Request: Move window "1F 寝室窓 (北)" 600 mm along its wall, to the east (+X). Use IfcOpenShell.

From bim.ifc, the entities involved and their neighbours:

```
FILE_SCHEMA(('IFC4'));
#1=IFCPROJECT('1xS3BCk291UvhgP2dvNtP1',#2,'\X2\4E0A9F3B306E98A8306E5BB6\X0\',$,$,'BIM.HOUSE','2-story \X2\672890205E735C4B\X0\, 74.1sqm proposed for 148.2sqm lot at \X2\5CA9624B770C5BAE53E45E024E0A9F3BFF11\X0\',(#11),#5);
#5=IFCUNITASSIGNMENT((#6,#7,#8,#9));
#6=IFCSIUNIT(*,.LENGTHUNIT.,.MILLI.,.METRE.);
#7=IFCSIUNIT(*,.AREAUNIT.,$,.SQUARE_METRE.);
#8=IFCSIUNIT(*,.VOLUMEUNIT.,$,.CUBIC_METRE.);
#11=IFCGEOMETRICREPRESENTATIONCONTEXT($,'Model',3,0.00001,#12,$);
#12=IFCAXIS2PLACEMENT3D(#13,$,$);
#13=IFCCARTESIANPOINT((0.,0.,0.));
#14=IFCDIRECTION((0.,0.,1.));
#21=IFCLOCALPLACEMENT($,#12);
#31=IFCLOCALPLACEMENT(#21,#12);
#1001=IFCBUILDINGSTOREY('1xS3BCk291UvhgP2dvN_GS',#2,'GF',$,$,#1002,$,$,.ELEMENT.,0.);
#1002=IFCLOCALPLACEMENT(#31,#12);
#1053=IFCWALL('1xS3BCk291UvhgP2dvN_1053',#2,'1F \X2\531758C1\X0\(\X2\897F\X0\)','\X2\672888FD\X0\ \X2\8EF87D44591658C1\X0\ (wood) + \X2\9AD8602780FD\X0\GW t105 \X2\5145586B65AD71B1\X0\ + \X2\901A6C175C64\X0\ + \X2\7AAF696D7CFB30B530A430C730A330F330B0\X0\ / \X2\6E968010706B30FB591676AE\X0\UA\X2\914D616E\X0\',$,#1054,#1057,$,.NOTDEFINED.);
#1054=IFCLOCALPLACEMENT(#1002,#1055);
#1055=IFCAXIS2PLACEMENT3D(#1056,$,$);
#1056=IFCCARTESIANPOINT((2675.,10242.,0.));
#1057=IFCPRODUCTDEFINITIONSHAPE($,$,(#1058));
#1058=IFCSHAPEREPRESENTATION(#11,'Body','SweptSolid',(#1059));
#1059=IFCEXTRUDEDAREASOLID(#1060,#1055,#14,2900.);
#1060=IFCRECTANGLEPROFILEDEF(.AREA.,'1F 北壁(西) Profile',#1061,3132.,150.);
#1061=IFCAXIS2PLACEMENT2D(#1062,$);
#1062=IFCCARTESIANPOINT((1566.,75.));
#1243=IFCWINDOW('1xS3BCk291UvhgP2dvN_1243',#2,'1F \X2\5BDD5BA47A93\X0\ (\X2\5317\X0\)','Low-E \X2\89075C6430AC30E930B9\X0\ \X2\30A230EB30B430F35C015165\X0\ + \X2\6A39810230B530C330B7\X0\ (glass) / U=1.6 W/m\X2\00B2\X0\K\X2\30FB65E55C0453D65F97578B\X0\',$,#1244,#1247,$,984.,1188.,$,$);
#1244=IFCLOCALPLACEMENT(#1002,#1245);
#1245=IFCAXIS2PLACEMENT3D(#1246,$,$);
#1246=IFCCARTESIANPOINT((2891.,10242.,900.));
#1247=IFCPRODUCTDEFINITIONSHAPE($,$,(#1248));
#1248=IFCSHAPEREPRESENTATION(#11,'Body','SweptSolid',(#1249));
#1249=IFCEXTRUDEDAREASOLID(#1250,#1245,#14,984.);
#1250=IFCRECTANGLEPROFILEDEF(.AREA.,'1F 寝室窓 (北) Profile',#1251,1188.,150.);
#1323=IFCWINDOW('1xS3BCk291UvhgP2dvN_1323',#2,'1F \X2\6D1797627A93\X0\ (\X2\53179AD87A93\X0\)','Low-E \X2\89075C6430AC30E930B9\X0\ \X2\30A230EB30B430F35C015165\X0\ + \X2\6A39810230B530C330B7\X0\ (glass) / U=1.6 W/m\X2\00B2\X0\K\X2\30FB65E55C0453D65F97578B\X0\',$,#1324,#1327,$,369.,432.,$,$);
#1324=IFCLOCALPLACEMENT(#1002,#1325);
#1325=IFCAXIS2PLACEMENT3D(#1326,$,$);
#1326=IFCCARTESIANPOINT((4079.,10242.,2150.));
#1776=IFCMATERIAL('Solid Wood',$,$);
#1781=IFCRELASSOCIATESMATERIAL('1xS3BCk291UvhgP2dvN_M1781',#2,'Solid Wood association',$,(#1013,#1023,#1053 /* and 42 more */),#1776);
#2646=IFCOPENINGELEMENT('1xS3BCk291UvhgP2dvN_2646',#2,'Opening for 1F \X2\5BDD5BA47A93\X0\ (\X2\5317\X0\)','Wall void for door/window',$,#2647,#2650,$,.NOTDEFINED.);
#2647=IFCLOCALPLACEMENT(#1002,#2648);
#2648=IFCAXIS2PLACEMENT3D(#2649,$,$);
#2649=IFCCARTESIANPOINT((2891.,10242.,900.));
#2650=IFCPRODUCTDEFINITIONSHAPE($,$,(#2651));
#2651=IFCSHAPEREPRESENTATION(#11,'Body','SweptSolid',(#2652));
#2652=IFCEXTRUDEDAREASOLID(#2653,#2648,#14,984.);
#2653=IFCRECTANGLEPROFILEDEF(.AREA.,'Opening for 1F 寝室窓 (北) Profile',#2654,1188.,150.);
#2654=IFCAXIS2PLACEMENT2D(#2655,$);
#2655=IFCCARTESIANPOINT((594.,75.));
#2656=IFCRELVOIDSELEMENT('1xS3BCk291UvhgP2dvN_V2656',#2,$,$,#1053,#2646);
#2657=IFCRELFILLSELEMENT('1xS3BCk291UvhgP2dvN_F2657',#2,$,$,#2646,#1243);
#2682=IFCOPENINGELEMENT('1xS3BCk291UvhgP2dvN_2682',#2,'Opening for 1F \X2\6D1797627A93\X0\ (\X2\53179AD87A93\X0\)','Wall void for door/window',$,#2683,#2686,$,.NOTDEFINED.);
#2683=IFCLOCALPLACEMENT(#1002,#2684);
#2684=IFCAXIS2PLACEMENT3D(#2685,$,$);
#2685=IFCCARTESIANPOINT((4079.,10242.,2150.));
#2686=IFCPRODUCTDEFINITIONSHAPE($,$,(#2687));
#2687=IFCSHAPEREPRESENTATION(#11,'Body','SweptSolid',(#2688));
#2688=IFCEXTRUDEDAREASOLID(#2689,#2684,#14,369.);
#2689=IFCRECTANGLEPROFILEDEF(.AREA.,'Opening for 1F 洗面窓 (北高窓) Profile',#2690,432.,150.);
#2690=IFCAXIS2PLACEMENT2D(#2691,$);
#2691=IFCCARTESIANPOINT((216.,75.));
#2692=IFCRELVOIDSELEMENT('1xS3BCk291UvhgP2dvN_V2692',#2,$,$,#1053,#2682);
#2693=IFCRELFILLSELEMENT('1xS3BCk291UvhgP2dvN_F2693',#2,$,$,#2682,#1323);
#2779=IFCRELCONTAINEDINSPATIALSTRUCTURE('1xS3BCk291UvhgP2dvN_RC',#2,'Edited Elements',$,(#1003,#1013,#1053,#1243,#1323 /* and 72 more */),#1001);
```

```python
import ifcopenshell
import ifcopenshell.api.geometry
import ifcopenshell.util.placement
import ifcopenshell.util.unit

model = ifcopenshell.open("bim.ifc")
unit_scale = ifcopenshell.util.unit.calculate_unit_scale(model)

window = model.by_id(1243)
opening = window.FillsVoids[0].RelatingOpeningElement
wall = opening.VoidsElements[0].RelatingBuildingElement

wall_matrix = ifcopenshell.util.placement.get_local_placement(wall.ObjectPlacement)
shift = wall_matrix[:3, 0] * 0.6 / unit_scale
before = ifcopenshell.util.placement.get_local_placement(window.ObjectPlacement)[:3, 3].copy()

# The window is not placed relative to its opening, so move both.
for product in (opening, window):
    matrix = ifcopenshell.util.placement.get_local_placement(product.ObjectPlacement)
    matrix[:3, 3] += shift
    ifcopenshell.api.geometry.edit_object_placement(model, product=product, matrix=matrix, is_si=False)

after = ifcopenshell.util.placement.get_local_placement(window.ObjectPlacement)[:3, 3]
print("window moved by", (after - before).round(3) + 0.0)

model.write("bim_updated.ifc")
```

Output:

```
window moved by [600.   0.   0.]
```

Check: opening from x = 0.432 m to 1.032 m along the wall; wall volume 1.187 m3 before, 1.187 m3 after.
